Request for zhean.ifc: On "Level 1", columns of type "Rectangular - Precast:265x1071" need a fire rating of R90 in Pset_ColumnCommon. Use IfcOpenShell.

First a look at what the model holds.

```python
import ifcopenshell
import ifcopenshell.util.element

model = ifcopenshell.open("zhean.ifc")
print(model.schema)
storey = next(s for s in model.by_type("IfcBuildingStorey") if s.Name == "Level 1")
columns = [e for e in ifcopenshell.util.element.get_decomposition(storey) if e.is_a("IfcColumn")]
seen = {}
for e in columns:
    element_type = ifcopenshell.util.element.get_type(e)
    key = (element_type.Name if element_type != e and element_type else None, ifcopenshell.util.element.get_pset(e, "Pset_ColumnCommon", "FireRating"))
    seen[key] = seen.get(key, 0) + 1
for (name, value), count in sorted(seen.items(), key=str):
    print(count, "x", name, "|", value)
```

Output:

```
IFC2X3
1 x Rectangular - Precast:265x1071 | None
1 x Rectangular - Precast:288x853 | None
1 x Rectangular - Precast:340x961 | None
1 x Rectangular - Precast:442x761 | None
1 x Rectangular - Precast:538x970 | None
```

```python
import ifcopenshell
import ifcopenshell.api.pset
import ifcopenshell.util.element

model = ifcopenshell.open("zhean.ifc")

storey = next(s for s in model.by_type("IfcBuildingStorey") if s.Name == "Level 1")
columns = [e for e in ifcopenshell.util.element.get_decomposition(storey) if e.is_a("IfcColumn")]

count = 0
for e in columns:
    element_type = ifcopenshell.util.element.get_type(e)
    if element_type in (None, e) or element_type.Name != "Rectangular - Precast:265x1071":
        continue
    # add_pset returns the element's existing set when there is one.
    pset = ifcopenshell.api.pset.add_pset(model, product=e, name="Pset_ColumnCommon")
    ifcopenshell.api.pset.edit_pset(model, pset=pset, properties={"FireRating": "R90"})
    count += 1

print(count, "columns updated")

model.write("zhean_edited.ifc")
```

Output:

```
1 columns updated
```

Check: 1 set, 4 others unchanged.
